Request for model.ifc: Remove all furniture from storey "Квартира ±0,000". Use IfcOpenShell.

First a look at what the model holds.

```python
import ifcopenshell
import ifcopenshell.util.element

model = ifcopenshell.open("model.ifc")
print(model.schema)
storey = next(s for s in model.by_type("IfcBuildingStorey") if s.Name == "Квартира ±0,000")
furniture = [e for e in ifcopenshell.util.element.get_decomposition(storey) if e.is_a("IfcFurnishingElement")]
seen = {}
for e in furniture:
    element_type = ifcopenshell.util.element.get_type(e)
    name = element_type.Name if element_type not in (None, e) else None
    seen[name] = seen.get(name, 0) + 1
for name, count in sorted(seen.items(), key=str):
    print(count, "x", name)
```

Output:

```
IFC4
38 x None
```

```python
import ifcopenshell
import ifcopenshell.api.root
import ifcopenshell.util.element

model = ifcopenshell.open("model.ifc")

storey = next(s for s in model.by_type("IfcBuildingStorey") if s.Name == "Квартира ±0,000")
furniture = [e for e in ifcopenshell.util.element.get_decomposition(storey) if e.is_a("IfcFurnishingElement")]

for e in furniture:
    ifcopenshell.api.root.remove_product(model, product=e)
print(len(furniture), "removed")

model.write("model_v2.ifc")
```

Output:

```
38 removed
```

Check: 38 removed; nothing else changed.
